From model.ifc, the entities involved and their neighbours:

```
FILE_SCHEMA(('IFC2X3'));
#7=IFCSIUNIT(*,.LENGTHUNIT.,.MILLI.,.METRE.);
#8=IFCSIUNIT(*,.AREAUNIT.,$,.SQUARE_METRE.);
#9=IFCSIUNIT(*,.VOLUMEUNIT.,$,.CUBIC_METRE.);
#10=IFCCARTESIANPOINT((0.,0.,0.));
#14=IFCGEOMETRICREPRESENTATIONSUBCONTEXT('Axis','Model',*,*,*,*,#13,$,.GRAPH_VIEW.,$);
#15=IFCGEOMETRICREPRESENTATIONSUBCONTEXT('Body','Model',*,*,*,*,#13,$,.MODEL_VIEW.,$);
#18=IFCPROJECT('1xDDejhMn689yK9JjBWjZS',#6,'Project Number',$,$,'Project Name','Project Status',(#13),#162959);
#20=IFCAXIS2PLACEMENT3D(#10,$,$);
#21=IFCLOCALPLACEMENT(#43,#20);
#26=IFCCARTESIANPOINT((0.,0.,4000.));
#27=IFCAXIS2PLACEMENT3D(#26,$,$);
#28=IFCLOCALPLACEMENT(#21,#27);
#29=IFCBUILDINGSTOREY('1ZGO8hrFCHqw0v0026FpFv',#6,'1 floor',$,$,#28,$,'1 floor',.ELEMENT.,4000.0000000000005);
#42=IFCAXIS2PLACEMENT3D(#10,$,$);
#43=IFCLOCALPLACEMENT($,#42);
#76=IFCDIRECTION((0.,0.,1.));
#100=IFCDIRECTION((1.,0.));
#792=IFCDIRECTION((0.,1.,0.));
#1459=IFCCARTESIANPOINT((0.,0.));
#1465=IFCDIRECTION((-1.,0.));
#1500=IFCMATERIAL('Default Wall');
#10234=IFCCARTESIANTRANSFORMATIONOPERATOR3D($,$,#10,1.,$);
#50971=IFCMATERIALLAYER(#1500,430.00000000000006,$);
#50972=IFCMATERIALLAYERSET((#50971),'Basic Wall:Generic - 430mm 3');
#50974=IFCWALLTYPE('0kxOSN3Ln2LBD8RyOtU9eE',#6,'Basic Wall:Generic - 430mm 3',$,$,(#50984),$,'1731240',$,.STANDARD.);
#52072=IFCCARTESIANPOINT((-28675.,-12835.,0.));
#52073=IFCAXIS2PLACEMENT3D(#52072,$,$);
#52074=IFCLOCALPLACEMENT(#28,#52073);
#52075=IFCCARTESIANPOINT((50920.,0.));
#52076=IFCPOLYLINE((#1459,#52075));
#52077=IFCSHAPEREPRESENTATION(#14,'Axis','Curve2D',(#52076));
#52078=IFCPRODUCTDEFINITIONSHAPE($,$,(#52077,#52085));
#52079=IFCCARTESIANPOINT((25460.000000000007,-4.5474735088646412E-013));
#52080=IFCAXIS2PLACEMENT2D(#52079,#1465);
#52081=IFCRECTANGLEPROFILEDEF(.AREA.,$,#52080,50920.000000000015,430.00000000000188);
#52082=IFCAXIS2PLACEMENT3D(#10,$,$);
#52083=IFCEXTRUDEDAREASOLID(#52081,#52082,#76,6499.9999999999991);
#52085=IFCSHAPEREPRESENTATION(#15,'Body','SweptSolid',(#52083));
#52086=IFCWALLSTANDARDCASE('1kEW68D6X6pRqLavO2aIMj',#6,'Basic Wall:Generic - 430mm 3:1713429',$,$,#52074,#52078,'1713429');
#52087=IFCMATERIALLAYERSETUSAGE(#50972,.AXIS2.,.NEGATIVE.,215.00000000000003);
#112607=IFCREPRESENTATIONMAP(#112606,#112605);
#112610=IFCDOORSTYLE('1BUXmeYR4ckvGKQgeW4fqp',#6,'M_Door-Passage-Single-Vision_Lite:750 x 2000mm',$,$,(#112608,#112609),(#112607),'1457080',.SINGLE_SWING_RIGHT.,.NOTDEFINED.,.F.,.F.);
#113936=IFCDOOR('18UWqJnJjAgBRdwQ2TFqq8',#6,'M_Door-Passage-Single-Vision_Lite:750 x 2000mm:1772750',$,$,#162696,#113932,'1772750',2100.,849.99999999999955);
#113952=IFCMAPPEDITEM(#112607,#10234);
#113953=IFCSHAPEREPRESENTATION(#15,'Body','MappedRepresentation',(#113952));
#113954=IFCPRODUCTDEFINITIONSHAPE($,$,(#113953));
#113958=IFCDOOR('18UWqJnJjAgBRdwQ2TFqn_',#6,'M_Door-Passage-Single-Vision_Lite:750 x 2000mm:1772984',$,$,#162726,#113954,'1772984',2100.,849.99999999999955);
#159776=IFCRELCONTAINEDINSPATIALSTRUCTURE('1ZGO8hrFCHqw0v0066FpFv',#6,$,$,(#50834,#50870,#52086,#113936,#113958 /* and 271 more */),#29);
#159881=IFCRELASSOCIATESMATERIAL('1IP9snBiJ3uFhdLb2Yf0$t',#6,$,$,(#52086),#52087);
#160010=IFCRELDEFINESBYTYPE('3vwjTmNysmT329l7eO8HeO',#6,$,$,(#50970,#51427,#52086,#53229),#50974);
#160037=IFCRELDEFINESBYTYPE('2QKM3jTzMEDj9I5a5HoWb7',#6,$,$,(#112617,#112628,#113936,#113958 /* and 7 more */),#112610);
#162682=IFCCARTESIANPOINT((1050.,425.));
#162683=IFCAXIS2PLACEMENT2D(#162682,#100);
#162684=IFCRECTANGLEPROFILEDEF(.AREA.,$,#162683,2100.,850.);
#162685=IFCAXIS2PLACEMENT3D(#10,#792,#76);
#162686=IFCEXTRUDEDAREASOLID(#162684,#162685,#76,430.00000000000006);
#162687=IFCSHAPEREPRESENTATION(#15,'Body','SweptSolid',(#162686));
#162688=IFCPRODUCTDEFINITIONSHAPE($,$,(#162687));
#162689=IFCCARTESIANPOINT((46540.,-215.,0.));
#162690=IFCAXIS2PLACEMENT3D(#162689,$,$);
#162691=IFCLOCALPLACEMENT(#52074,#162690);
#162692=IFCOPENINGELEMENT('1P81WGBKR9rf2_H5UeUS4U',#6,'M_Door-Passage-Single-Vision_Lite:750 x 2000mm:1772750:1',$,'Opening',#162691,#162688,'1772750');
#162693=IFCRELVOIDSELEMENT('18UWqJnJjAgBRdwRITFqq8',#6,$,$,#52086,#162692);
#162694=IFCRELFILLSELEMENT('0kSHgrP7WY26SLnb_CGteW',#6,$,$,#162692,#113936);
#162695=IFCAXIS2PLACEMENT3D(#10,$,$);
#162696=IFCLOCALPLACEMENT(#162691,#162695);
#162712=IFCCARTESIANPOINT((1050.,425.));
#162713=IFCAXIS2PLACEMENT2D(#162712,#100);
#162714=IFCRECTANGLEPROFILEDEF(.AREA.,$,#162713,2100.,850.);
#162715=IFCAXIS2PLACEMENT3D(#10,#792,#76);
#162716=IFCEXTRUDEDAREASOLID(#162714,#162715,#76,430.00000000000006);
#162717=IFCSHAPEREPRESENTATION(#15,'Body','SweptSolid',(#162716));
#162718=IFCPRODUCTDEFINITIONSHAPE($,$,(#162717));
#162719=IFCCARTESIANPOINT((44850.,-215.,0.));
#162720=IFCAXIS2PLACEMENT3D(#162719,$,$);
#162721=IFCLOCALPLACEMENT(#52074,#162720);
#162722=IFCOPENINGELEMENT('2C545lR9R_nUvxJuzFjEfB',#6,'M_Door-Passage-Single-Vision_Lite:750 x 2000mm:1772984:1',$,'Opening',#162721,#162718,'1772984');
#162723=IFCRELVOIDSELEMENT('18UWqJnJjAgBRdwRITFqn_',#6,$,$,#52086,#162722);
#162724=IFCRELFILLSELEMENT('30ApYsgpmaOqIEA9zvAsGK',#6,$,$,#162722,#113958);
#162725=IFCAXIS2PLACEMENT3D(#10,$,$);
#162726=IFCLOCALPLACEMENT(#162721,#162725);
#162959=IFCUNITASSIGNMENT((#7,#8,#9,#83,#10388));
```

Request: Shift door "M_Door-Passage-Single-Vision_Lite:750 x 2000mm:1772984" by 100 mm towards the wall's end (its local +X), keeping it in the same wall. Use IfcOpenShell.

```python
import ifcopenshell
import ifcopenshell.api.geometry
import ifcopenshell.util.placement

model = ifcopenshell.open("model.ifc")

door = model.by_guid("18UWqJnJjAgBRdwQ2TFqn_")
opening = door.FillsVoids[0].RelatingOpeningElement
wall = opening.VoidsElements[0].RelatingBuildingElement

wall_matrix = ifcopenshell.util.placement.get_local_placement(wall.ObjectPlacement)
shift = wall_matrix[:3, 0] * 100.0
before = ifcopenshell.util.placement.get_local_placement(door.ObjectPlacement)[:3, 3].copy()

# The door is placed relative to its opening, so it follows when the opening moves.
matrix = ifcopenshell.util.placement.get_local_placement(opening.ObjectPlacement)
matrix[:3, 3] += shift
ifcopenshell.api.geometry.edit_object_placement(
    model, product=opening, matrix=matrix, is_si=False, should_transform_children=True
)

after = ifcopenshell.util.placement.get_local_placement(door.ObjectPlacement)[:3, 3]
print("door moved by", (after - before).round(3) + 0.0)

model.write("model_rev.ifc")
```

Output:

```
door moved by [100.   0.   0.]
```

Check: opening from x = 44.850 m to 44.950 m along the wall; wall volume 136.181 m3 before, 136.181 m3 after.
